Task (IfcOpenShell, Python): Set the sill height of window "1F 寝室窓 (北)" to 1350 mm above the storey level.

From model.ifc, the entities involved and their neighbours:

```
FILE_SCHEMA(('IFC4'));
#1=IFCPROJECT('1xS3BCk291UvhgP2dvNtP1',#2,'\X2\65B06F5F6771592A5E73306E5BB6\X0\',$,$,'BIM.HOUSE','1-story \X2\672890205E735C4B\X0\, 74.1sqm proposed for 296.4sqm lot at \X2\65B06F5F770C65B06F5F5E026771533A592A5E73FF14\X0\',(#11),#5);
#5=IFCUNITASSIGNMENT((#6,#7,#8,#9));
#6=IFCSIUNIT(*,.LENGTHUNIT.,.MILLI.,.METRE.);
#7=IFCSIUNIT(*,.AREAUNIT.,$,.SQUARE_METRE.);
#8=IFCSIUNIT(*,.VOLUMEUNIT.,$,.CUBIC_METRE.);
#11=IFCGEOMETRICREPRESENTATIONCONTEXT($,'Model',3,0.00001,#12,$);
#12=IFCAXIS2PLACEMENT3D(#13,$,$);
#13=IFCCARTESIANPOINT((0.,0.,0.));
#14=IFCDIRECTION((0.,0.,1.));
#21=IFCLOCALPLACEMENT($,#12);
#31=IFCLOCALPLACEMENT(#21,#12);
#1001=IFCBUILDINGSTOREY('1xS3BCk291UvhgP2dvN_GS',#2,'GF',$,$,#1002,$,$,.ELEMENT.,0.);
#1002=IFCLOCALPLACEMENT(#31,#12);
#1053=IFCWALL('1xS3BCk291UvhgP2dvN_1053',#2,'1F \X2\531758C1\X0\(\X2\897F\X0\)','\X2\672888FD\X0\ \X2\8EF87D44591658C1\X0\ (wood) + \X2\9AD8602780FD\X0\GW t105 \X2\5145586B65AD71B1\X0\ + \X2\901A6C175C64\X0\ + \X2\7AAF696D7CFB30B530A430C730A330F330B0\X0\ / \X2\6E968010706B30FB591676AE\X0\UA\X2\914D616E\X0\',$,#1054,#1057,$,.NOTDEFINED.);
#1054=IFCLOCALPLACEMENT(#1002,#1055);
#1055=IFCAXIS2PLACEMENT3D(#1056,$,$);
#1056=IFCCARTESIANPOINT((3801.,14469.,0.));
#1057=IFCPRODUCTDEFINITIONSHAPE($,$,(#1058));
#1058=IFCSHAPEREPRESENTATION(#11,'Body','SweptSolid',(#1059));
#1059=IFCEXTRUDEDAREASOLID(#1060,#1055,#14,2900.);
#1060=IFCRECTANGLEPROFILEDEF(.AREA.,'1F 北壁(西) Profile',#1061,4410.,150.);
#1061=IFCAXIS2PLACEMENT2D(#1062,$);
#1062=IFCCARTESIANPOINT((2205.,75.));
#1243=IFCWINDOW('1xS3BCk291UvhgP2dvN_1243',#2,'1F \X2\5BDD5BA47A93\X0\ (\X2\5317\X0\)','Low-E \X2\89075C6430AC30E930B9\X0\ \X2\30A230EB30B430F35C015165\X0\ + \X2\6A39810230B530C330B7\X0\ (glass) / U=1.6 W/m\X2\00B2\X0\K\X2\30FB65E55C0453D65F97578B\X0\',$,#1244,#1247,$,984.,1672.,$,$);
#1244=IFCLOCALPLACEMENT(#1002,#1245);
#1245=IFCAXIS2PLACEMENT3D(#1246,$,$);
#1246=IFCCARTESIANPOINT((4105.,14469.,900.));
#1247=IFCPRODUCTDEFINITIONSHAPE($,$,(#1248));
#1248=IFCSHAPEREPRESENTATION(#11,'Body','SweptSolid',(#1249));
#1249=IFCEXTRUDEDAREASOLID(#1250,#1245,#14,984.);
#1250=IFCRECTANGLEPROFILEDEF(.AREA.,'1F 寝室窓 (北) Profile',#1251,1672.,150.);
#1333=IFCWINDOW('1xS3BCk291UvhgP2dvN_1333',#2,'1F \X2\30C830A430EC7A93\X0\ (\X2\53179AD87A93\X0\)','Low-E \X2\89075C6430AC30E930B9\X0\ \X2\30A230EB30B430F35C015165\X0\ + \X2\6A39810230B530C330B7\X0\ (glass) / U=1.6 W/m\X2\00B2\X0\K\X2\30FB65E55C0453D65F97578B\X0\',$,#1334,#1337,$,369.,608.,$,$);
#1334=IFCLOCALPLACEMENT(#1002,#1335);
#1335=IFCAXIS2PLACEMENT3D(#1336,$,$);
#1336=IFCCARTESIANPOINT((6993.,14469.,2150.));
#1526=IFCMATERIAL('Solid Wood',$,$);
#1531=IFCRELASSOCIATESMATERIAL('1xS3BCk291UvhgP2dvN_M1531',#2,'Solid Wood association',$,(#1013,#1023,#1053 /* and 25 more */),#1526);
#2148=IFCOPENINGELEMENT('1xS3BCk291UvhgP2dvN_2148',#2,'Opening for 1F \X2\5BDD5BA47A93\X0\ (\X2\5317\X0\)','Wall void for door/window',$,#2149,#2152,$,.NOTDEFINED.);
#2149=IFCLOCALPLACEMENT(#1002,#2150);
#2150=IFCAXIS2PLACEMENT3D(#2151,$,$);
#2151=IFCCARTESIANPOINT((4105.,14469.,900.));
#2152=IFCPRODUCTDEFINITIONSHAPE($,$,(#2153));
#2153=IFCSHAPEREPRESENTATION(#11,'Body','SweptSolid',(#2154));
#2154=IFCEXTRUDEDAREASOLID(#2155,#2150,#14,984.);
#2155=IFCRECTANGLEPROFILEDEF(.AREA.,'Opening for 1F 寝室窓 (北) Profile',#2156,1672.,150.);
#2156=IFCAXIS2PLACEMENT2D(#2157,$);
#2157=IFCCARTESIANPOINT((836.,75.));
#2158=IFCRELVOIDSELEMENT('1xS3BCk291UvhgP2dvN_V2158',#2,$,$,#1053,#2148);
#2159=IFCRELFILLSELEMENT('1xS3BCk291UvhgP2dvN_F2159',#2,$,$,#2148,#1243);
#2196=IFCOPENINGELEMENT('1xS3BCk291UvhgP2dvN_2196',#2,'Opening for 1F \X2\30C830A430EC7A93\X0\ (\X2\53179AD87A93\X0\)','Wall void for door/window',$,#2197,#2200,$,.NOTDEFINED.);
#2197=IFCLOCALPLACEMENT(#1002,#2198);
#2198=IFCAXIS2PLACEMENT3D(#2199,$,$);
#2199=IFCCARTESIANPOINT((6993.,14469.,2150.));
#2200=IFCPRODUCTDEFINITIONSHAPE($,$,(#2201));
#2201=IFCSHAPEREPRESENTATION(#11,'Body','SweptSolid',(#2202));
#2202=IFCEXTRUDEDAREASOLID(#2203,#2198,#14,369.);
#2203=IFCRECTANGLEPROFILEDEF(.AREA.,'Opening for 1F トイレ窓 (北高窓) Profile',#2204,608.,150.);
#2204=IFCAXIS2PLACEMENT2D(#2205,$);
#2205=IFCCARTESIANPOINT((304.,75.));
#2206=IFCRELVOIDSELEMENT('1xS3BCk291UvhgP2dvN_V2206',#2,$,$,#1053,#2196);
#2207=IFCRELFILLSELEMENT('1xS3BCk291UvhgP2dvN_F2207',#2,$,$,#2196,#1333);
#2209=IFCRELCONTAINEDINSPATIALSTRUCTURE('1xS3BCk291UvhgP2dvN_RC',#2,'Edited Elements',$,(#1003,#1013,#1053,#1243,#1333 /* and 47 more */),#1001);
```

```python
import numpy as np
import ifcopenshell
import ifcopenshell.api.geometry
import ifcopenshell.geom
import ifcopenshell.util.element
import ifcopenshell.util.placement
import ifcopenshell.util.shape
import ifcopenshell.util.unit

model = ifcopenshell.open("model.ifc")
unit_scale = ifcopenshell.util.unit.calculate_unit_scale(model)

window = model.by_guid("1xS3BCk291UvhgP2dvN_1243")
opening = window.FillsVoids[0].RelatingOpeningElement
storey = ifcopenshell.util.element.get_container(window, ifc_class="IfcBuildingStorey")
level = ifcopenshell.util.placement.get_local_placement(storey.ObjectPlacement)[2, 3]

# The opening's origin need not be at the sill, so measure its lowest point.
shape = ifcopenshell.geom.create_shape(ifcopenshell.geom.settings(), opening)
bottom = ifcopenshell.util.shape.get_shape_bottom_elevation(shape, shape.geometry) / unit_scale
dz = level + 1.35 / unit_scale - bottom

shift = np.array([0.0, 0.0, dz])
# The window is not placed relative to its opening, so move both.
for product in (opening, window):
    matrix = ifcopenshell.util.placement.get_local_placement(product.ObjectPlacement)
    matrix[:3, 3] += shift
    ifcopenshell.api.geometry.edit_object_placement(model, product=product, matrix=matrix, is_si=False)

print(f"moved by {dz * unit_scale:+.3f} m")

model.write("model_rev.ifc")
```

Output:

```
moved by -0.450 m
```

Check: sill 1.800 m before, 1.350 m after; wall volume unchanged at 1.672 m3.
